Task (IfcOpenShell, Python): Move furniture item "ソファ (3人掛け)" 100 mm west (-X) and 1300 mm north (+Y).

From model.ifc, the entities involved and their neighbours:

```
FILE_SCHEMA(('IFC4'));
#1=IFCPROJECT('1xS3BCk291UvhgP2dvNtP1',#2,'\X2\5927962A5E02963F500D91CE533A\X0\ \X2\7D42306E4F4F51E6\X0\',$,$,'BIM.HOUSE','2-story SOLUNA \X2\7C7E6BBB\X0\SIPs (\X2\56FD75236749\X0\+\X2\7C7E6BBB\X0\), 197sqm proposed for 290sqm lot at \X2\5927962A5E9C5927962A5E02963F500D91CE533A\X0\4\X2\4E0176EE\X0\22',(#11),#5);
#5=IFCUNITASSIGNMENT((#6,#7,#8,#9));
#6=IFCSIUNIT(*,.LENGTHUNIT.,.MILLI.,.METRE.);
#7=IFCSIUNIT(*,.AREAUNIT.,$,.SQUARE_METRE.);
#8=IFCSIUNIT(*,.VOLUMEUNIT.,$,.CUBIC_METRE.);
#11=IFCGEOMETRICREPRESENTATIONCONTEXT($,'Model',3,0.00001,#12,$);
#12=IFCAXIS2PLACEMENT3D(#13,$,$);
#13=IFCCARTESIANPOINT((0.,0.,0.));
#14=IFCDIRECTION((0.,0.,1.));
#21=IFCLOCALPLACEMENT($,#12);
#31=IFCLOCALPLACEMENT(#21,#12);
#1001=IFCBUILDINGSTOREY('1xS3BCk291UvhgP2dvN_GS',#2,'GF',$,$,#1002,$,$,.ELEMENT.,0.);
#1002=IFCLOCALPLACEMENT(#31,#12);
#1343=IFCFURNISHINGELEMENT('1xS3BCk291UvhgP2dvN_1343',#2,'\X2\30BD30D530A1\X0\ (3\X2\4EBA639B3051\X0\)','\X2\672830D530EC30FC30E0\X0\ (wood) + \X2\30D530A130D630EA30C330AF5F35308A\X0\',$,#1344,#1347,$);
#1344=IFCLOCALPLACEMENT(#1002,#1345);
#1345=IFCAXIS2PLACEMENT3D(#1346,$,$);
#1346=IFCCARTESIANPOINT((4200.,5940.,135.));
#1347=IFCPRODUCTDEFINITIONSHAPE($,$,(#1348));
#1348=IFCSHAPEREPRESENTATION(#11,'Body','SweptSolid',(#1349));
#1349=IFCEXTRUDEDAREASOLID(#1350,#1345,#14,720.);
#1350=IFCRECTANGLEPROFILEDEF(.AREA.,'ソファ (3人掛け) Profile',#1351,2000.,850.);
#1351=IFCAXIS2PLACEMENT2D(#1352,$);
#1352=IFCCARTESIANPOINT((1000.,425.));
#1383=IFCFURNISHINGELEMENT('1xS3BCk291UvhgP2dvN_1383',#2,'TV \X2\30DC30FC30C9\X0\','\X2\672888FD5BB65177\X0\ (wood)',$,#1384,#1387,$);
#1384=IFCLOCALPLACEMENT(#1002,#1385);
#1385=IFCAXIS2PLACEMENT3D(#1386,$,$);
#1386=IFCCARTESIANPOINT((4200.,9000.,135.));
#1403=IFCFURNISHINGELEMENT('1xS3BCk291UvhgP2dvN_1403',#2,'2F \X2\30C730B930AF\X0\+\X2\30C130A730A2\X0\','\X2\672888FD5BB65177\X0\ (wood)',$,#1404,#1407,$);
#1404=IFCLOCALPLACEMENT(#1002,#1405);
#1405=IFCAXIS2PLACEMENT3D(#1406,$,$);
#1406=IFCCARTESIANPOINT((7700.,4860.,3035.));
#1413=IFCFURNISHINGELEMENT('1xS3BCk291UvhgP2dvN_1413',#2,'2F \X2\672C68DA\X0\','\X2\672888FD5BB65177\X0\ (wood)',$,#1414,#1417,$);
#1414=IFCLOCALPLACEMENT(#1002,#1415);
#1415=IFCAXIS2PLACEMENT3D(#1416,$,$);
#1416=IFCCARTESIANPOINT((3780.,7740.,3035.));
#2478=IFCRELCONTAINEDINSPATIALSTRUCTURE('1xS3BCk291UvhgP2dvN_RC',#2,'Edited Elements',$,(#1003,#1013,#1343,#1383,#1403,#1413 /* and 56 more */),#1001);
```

```python
import ifcopenshell
import ifcopenshell.api.geometry
import ifcopenshell.util.placement
import ifcopenshell.util.unit

model = ifcopenshell.open("model.ifc")
unit_scale = ifcopenshell.util.unit.calculate_unit_scale(model)

item = model.by_guid("1xS3BCk291UvhgP2dvN_1343")
matrix = ifcopenshell.util.placement.get_local_placement(item.ObjectPlacement)
matrix[0, 3] -= 0.1 / unit_scale
matrix[1, 3] += 1.3 / unit_scale
ifcopenshell.api.geometry.edit_object_placement(model, product=item, matrix=matrix, is_si=False)

print(ifcopenshell.util.placement.get_local_placement(item.ObjectPlacement).round(3) + 0.0)

model.write("model-out.ifc")
```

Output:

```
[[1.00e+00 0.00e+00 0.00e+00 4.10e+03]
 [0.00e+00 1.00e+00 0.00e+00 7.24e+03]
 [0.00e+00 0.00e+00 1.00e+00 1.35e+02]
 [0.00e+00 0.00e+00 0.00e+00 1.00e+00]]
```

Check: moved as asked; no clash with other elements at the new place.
